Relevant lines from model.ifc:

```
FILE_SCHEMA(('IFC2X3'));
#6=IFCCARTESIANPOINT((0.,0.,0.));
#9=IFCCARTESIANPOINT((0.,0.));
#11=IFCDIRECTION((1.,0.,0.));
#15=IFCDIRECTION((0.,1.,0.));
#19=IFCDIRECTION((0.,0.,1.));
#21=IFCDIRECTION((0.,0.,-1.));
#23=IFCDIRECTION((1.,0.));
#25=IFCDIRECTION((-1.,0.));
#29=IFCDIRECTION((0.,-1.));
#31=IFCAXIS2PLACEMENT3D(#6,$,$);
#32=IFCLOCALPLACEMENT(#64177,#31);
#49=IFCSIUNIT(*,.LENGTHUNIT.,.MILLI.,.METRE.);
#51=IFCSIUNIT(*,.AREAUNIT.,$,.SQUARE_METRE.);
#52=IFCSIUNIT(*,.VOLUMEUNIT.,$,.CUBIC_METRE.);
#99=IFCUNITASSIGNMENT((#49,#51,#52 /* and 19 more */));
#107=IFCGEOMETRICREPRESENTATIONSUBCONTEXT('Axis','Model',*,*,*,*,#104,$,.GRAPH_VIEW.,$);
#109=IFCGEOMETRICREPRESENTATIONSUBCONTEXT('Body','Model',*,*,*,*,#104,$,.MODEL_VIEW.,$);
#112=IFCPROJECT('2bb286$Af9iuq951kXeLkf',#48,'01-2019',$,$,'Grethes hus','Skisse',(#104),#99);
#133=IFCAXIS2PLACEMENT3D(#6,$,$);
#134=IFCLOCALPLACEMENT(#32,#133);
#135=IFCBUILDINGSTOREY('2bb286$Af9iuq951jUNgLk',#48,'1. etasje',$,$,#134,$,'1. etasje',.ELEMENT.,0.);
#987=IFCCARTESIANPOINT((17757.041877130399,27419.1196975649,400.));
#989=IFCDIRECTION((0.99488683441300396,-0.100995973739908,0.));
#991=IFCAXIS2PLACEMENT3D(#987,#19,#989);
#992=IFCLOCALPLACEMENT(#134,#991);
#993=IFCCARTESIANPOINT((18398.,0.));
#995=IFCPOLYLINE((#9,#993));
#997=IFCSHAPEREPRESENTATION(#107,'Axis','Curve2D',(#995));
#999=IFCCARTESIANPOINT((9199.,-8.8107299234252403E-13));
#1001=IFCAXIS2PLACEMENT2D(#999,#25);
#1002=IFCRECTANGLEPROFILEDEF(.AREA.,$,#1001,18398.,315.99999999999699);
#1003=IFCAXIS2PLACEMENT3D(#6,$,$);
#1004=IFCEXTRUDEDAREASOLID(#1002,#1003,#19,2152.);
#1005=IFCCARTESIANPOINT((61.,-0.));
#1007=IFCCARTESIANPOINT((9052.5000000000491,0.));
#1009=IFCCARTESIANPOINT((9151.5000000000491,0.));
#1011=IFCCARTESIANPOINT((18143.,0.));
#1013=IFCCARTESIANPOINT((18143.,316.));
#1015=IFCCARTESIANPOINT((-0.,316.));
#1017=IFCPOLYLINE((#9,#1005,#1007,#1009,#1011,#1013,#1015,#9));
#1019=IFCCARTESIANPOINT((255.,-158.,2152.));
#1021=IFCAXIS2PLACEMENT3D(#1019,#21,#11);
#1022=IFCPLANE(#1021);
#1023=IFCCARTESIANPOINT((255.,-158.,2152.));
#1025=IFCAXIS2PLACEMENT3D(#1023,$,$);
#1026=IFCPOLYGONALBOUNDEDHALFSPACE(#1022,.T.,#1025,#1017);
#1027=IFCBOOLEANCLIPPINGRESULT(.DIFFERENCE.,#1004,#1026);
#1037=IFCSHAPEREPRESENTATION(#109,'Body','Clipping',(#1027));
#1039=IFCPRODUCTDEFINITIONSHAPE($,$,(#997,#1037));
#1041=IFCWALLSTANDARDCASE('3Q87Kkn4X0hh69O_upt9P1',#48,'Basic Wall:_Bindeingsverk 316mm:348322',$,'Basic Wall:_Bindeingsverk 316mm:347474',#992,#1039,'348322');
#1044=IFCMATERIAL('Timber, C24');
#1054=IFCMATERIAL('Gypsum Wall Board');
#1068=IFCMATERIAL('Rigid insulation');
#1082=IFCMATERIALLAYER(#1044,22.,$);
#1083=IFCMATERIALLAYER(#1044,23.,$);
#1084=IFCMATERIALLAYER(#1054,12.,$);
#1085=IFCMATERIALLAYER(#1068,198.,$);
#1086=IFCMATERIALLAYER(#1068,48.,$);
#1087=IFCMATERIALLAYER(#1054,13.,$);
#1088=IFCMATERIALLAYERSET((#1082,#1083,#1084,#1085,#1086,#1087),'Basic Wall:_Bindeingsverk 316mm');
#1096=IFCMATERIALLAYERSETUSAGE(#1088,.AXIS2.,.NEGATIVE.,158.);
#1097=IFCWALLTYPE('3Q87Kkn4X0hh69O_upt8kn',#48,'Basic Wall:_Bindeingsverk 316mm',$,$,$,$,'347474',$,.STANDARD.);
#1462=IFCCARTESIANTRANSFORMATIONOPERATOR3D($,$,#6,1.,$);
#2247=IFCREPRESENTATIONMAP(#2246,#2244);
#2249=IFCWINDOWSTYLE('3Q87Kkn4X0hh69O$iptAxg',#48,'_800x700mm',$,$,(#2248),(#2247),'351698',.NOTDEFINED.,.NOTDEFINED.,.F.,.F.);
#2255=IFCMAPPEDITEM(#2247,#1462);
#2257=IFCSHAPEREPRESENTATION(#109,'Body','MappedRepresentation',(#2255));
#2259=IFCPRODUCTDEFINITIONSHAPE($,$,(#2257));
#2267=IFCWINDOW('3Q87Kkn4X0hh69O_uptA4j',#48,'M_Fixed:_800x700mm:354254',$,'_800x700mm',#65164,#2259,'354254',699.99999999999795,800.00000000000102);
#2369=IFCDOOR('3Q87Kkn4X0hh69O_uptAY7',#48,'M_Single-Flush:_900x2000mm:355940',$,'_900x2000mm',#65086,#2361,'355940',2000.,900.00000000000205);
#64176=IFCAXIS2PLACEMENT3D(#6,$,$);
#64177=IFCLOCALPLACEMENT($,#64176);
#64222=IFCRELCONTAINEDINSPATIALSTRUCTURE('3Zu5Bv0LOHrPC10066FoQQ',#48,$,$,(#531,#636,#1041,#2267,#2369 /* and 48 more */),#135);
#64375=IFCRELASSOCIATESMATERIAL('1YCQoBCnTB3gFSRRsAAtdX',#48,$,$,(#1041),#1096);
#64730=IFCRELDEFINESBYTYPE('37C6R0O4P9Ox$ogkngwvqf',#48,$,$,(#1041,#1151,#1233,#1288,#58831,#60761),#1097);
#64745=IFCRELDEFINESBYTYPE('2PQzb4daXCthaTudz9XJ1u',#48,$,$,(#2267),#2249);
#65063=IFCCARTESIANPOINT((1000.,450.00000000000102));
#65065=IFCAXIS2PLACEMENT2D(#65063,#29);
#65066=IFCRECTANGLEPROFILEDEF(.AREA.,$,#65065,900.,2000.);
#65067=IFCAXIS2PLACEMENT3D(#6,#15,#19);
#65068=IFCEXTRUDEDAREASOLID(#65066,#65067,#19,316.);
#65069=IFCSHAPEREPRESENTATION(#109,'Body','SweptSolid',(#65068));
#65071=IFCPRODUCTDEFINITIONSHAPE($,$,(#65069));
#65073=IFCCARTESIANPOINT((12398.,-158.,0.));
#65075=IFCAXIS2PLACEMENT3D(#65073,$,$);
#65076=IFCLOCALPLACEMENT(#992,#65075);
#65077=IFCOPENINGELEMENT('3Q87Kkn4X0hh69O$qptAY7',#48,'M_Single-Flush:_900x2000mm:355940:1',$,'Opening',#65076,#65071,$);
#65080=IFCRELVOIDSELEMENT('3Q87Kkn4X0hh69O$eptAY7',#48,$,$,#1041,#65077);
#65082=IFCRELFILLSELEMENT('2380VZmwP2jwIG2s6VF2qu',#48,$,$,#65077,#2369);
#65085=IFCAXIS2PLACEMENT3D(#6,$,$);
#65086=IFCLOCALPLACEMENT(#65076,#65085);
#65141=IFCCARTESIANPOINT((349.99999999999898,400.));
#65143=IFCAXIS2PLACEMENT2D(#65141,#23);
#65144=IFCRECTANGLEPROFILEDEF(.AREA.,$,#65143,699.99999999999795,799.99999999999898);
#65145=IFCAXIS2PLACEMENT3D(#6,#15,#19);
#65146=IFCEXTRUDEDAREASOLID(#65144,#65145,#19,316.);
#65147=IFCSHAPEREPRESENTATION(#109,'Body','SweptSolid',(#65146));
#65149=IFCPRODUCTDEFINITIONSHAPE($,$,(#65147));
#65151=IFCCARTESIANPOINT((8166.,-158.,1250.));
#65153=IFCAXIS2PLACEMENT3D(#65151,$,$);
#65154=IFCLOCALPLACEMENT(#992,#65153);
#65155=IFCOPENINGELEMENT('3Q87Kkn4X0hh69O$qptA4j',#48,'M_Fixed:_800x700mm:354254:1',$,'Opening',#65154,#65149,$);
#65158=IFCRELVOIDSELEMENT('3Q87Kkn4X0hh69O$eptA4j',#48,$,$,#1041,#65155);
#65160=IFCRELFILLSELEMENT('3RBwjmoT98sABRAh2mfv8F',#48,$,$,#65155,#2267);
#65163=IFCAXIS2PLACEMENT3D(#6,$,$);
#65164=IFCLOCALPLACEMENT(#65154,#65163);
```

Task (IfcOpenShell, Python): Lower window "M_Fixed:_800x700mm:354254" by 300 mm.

```python
import numpy as np
import ifcopenshell
import ifcopenshell.api.geometry
import ifcopenshell.util.placement
import ifcopenshell.util.unit

model = ifcopenshell.open("model.ifc")
unit_scale = ifcopenshell.util.unit.calculate_unit_scale(model)

window = model.by_id(2267)
opening = window.FillsVoids[0].RelatingOpeningElement
dz = -0.3 / unit_scale

shift = np.array([0.0, 0.0, dz])
# The window is placed relative to its opening, so it follows when the opening moves.
matrix = ifcopenshell.util.placement.get_local_placement(opening.ObjectPlacement)
matrix[:3, 3] += shift
ifcopenshell.api.geometry.edit_object_placement(
    model, product=opening, matrix=matrix, is_si=False, should_transform_children=True
)

print(f"moved by {dz * unit_scale:+.3f} m")

model.write("model_rev.ifc")
```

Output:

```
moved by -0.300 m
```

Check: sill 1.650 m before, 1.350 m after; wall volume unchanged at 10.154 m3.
